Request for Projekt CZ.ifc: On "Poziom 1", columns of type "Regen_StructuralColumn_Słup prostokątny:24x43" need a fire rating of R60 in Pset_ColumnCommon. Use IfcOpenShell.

First a look at what the model holds.

```python
import ifcopenshell
import ifcopenshell.util.element

model = ifcopenshell.open("Projekt CZ.ifc")
print(model.schema)
storey = next(s for s in model.by_type("IfcBuildingStorey") if s.Name == "Poziom 1")
columns = [e for e in ifcopenshell.util.element.get_decomposition(storey) if e.is_a("IfcColumn")]
seen = {}
for e in columns:
    element_type = ifcopenshell.util.element.get_type(e)
    key = (element_type.Name if element_type != e and element_type else None, ifcopenshell.util.element.get_pset(e, "Pset_ColumnCommon", "FireRating"))
    seen[key] = seen.get(key, 0) + 1
for (name, value), count in sorted(seen.items(), key=str):
    print(count, "x", name, "|", value)
```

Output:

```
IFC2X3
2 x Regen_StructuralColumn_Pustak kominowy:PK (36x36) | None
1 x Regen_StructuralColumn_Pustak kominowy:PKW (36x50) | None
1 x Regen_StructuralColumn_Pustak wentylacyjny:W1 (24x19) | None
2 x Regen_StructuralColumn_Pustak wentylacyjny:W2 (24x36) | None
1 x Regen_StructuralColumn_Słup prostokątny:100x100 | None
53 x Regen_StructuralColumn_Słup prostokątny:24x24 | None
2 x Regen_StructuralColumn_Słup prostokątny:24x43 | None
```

```python
import ifcopenshell
import ifcopenshell.api.pset
import ifcopenshell.util.element

model = ifcopenshell.open("Projekt CZ.ifc")

storey = next(s for s in model.by_type("IfcBuildingStorey") if s.Name == "Poziom 1")
columns = [e for e in ifcopenshell.util.element.get_decomposition(storey) if e.is_a("IfcColumn")]

count = 0
for e in columns:
    element_type = ifcopenshell.util.element.get_type(e)
    if element_type in (None, e) or element_type.Name != "Regen_StructuralColumn_Słup prostokątny:24x43":
        continue
    # add_pset returns the element's existing set when there is one.
    pset = ifcopenshell.api.pset.add_pset(model, product=e, name="Pset_ColumnCommon")
    ifcopenshell.api.pset.edit_pset(model, pset=pset, properties={"FireRating": "R60"})
    count += 1

print(count, "columns updated")

model.write("Projekt CZ-out.ifc")
```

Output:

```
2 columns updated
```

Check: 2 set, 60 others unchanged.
